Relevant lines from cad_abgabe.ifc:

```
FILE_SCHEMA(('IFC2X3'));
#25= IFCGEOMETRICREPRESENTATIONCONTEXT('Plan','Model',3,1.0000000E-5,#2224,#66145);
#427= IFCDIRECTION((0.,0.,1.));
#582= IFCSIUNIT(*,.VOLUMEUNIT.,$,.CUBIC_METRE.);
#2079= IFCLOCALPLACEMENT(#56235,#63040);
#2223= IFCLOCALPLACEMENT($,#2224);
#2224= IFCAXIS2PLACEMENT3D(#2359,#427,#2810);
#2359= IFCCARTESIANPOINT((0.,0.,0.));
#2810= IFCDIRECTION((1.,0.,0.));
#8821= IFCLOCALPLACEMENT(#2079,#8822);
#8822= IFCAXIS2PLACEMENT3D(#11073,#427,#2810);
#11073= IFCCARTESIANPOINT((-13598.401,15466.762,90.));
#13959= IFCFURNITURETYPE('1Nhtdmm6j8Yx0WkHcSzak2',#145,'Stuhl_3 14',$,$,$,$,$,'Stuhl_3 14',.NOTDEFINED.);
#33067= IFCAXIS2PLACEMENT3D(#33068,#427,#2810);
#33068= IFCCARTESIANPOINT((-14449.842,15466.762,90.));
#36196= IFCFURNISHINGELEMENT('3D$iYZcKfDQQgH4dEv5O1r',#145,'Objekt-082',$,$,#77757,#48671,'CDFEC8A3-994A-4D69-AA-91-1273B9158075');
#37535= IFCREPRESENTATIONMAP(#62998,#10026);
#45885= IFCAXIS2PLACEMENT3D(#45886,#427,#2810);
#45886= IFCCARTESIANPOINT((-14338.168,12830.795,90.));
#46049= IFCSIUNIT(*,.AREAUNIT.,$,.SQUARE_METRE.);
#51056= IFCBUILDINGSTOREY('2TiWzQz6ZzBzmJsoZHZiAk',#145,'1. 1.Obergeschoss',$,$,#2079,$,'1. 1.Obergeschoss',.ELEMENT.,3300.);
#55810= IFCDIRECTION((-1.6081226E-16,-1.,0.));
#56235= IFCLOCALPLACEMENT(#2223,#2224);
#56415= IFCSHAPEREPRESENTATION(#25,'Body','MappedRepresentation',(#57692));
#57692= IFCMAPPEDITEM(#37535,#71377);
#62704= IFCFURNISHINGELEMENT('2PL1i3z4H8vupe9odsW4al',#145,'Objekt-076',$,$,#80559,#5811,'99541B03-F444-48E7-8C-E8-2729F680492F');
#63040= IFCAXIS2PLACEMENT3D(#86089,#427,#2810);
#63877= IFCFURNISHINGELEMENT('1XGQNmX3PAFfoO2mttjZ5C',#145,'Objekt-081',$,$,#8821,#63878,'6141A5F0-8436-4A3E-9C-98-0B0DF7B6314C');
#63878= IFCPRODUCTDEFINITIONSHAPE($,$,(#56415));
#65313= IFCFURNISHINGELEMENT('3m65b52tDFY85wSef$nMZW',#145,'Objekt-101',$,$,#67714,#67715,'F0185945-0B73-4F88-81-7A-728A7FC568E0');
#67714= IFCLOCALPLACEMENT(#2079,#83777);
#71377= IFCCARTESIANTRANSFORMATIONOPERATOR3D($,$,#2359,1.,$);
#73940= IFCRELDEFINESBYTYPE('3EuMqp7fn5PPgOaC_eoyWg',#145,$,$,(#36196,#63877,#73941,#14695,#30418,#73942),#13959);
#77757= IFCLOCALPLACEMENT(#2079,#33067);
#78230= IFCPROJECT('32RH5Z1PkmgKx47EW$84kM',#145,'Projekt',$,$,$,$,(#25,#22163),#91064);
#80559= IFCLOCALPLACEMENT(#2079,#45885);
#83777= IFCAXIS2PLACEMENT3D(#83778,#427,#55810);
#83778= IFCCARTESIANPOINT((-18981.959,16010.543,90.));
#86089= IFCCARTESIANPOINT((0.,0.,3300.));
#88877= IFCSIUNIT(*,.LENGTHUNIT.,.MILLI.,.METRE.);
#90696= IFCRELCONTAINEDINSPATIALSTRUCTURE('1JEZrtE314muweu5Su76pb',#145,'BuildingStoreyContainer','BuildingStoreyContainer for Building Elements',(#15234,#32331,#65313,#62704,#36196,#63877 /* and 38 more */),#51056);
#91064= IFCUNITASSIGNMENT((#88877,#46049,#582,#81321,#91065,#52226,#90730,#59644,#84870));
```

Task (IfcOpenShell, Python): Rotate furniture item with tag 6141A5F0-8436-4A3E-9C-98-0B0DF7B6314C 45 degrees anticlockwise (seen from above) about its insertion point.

```python
import ifcopenshell
import ifcopenshell.api.geometry
import ifcopenshell.util.placement

model = ifcopenshell.open("cad_abgabe.ifc")

item = model.by_guid("1XGQNmX3PAFfoO2mttjZ5C")
matrix = ifcopenshell.util.placement.get_local_placement(item.ObjectPlacement)
matrix = matrix @ ifcopenshell.util.placement.rotation(45, "Z")
ifcopenshell.api.geometry.edit_object_placement(model, product=item, matrix=matrix, is_si=False)

print(ifcopenshell.util.placement.get_local_placement(item.ObjectPlacement).round(3) + 0.0)

model.write("cad_abgabe_v2.ifc")
```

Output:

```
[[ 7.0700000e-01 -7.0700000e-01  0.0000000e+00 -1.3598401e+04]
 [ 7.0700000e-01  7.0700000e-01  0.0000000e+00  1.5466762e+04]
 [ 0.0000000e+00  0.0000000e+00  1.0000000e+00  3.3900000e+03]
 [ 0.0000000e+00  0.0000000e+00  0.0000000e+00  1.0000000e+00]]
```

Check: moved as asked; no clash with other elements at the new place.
